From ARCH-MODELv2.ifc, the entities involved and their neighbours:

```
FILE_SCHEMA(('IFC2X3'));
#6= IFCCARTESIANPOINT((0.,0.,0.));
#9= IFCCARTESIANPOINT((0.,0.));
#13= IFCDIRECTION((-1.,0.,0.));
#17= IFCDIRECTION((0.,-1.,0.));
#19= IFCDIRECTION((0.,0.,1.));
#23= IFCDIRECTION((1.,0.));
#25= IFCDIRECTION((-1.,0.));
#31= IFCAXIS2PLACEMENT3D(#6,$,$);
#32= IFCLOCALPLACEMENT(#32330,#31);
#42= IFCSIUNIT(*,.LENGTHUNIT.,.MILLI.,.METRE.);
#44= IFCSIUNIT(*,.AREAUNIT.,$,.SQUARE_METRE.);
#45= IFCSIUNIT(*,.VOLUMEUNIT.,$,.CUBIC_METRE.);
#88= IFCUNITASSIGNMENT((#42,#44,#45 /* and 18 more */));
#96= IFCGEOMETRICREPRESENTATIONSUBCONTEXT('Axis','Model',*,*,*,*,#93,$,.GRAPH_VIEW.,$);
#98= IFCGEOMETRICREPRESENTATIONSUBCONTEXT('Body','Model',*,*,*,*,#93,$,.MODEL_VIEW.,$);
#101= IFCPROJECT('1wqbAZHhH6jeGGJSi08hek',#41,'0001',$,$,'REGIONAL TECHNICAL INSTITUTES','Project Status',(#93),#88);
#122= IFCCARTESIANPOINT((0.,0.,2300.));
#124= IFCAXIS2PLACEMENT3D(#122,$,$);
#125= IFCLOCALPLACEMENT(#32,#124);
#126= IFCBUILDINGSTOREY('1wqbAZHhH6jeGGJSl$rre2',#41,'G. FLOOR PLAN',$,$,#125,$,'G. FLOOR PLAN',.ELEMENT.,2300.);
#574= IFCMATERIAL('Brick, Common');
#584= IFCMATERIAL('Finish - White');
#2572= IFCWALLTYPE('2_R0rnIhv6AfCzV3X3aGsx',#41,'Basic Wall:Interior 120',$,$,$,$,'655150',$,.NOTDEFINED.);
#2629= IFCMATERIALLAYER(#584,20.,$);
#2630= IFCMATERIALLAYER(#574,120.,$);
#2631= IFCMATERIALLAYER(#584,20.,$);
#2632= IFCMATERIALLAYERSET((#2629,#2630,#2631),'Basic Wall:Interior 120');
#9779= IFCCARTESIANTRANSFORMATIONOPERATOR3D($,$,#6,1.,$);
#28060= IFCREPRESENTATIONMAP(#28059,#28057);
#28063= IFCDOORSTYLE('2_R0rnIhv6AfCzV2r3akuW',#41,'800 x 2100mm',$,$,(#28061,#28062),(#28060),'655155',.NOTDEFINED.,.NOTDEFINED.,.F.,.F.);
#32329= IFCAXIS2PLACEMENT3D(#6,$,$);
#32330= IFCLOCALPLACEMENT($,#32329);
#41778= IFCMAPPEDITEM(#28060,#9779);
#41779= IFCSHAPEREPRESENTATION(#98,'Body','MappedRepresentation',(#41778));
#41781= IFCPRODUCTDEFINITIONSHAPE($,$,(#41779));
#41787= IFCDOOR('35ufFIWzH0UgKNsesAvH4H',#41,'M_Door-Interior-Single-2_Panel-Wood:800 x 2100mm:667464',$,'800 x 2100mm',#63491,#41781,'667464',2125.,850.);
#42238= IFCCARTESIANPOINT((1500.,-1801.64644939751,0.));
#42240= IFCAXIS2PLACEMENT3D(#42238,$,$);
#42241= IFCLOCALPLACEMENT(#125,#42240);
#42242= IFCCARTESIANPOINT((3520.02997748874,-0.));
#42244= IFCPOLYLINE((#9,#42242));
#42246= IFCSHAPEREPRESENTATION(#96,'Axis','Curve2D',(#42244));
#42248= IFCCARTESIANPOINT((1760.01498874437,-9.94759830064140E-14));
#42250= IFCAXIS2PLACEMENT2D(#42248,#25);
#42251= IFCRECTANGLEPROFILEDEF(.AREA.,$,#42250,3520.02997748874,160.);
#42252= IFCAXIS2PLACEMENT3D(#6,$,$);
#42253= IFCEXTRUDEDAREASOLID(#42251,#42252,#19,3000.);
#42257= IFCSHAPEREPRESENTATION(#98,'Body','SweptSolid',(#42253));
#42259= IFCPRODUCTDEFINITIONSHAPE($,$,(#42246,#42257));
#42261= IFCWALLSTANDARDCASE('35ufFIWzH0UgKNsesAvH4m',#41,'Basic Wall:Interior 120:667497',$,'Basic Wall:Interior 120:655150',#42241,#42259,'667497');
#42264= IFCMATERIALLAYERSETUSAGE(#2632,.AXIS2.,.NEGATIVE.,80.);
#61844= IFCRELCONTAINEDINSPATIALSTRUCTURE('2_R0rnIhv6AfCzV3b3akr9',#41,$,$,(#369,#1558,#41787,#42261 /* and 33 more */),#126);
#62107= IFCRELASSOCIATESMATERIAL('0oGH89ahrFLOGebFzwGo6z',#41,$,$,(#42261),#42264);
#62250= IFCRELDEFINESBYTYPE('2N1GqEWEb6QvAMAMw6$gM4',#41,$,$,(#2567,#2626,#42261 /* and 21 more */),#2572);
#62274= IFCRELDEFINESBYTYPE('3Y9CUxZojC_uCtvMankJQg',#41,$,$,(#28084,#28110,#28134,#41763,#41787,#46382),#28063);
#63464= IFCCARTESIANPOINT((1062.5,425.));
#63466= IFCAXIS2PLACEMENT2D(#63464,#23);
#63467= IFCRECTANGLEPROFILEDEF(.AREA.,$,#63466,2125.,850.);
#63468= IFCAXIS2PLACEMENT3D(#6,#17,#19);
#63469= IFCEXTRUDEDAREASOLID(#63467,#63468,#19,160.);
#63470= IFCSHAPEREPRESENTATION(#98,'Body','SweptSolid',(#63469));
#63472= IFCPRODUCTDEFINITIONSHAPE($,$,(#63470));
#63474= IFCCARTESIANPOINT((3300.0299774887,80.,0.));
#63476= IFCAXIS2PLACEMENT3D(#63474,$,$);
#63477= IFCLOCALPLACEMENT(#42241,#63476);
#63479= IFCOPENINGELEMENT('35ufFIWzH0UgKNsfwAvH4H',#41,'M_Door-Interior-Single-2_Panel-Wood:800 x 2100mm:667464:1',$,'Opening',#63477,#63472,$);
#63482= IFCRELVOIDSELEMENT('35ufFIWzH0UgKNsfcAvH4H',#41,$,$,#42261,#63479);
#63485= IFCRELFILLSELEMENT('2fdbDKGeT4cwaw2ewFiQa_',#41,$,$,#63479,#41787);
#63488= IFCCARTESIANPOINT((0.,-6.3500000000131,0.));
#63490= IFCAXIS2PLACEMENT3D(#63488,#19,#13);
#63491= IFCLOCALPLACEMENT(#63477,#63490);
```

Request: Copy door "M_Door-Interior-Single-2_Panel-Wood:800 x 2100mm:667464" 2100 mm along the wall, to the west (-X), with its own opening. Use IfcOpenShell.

```python
import ifcopenshell
import ifcopenshell.api.feature
import ifcopenshell.api.geometry
import ifcopenshell.api.root
import ifcopenshell.geom
import ifcopenshell.util.element
import ifcopenshell.util.placement
import ifcopenshell.util.shape

model = ifcopenshell.open("ARCH-MODELv2.ifc")
settings = ifcopenshell.geom.settings()


def volume(element):
    """Net volume in cubic metres, openings subtracted."""
    shape = ifcopenshell.geom.create_shape(settings, element)
    return ifcopenshell.util.shape.get_volume(shape.geometry)


def reuse_history(source, copy):
    """copy_class also copies each property set's owner history, people and application; keep the originals."""
    for rel in copy.IsDefinedBy:
        if rel.is_a("IfcRelDefinesByProperties") and (history := rel.RelatingPropertyDefinition.OwnerHistory):
            rel.RelatingPropertyDefinition.OwnerHistory = source.OwnerHistory
            ifcopenshell.util.element.remove_deep2(model, history)


door = model.by_guid("35ufFIWzH0UgKNsesAvH4H")
opening = door.FillsVoids[0].RelatingOpeningElement
wall = opening.VoidsElements[0].RelatingBuildingElement
before = volume(wall)
shift = ifcopenshell.util.placement.get_local_placement(wall.ObjectPlacement)[:3, 0] * -2100.0

# copy_class copies the void relationship, type, container and properties, but no geometry.
new_opening = ifcopenshell.api.root.copy_class(model, product=opening)
new_opening.Representation = ifcopenshell.util.element.copy_deep(
    model, opening.Representation, exclude=["IfcGeometricRepresentationContext", "IfcRepresentationMap"]
)
new_opening.Name = "M_Door-Interior-Single-2_Panel-Wood:800 x 2100mm"
new_door = ifcopenshell.api.root.copy_class(model, product=door)
new_door.Representation = ifcopenshell.util.element.copy_deep(
    model, door.Representation, exclude=["IfcGeometricRepresentationContext", "IfcRepresentationMap"]
)
new_door.Name = "M_Door-Interior-Single-2_Panel-Wood:800 x 2100mm"
new_door.Tag = None
reuse_history(door, new_door)
fills = ifcopenshell.api.feature.add_filling(model, opening=new_opening, element=new_door)
fills.OwnerHistory = new_door.OwnerHistory  # required in IFC2X3

for old, new in ((opening, new_opening), (door, new_door)):
    matrix = ifcopenshell.util.placement.get_local_placement(old.ObjectPlacement)
    matrix[:3, 3] += shift
    ifcopenshell.api.geometry.edit_object_placement(model, product=new, matrix=matrix, is_si=False)

after = volume(wall)

print(f"wall volume {before:.3f} -> {after:.3f} m3")

model.write("ARCH-MODELv2-out.ifc")
```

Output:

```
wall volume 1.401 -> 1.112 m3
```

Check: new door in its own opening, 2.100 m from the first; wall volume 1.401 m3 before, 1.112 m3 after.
